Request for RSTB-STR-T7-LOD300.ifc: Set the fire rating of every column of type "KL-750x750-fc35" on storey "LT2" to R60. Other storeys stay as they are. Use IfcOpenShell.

First a look at what the model holds.

```python
import ifcopenshell
import ifcopenshell.util.element

model = ifcopenshell.open("RSTB-STR-T7-LOD300.ifc")
print(model.schema)
storey = next(s for s in model.by_type("IfcBuildingStorey") if s.Name == "LT2")
columns = [e for e in ifcopenshell.util.element.get_decomposition(storey) if e.is_a("IfcColumn")]
seen = {}
for e in columns:
    element_type = ifcopenshell.util.element.get_type(e)
    key = (element_type.Name if element_type != e and element_type else None, ifcopenshell.util.element.get_pset(e, "Pset_ColumnCommon", "FireRating"))
    seen[key] = seen.get(key, 0) + 1
for (name, value), count in sorted(seen.items(), key=str):
    print(count, "x", name, "|", value)
```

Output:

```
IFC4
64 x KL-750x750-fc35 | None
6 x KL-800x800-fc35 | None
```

```python
import ifcopenshell
import ifcopenshell.api.pset
import ifcopenshell.util.element

model = ifcopenshell.open("RSTB-STR-T7-LOD300.ifc")

storey = next(s for s in model.by_type("IfcBuildingStorey") if s.Name == "LT2")
columns = [e for e in ifcopenshell.util.element.get_decomposition(storey) if e.is_a("IfcColumn")]

count = 0
for e in columns:
    element_type = ifcopenshell.util.element.get_type(e)
    if element_type in (None, e) or element_type.Name != "KL-750x750-fc35":
        continue
    # add_pset returns the element's existing set when there is one.
    pset = ifcopenshell.api.pset.add_pset(model, product=e, name="Pset_ColumnCommon")
    ifcopenshell.api.pset.edit_pset(model, pset=pset, properties={"FireRating": "R60"})
    count += 1

print(count, "columns updated")

model.write("RSTB-STR-T7-LOD300_edited.ifc")
```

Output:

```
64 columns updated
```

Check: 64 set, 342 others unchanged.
